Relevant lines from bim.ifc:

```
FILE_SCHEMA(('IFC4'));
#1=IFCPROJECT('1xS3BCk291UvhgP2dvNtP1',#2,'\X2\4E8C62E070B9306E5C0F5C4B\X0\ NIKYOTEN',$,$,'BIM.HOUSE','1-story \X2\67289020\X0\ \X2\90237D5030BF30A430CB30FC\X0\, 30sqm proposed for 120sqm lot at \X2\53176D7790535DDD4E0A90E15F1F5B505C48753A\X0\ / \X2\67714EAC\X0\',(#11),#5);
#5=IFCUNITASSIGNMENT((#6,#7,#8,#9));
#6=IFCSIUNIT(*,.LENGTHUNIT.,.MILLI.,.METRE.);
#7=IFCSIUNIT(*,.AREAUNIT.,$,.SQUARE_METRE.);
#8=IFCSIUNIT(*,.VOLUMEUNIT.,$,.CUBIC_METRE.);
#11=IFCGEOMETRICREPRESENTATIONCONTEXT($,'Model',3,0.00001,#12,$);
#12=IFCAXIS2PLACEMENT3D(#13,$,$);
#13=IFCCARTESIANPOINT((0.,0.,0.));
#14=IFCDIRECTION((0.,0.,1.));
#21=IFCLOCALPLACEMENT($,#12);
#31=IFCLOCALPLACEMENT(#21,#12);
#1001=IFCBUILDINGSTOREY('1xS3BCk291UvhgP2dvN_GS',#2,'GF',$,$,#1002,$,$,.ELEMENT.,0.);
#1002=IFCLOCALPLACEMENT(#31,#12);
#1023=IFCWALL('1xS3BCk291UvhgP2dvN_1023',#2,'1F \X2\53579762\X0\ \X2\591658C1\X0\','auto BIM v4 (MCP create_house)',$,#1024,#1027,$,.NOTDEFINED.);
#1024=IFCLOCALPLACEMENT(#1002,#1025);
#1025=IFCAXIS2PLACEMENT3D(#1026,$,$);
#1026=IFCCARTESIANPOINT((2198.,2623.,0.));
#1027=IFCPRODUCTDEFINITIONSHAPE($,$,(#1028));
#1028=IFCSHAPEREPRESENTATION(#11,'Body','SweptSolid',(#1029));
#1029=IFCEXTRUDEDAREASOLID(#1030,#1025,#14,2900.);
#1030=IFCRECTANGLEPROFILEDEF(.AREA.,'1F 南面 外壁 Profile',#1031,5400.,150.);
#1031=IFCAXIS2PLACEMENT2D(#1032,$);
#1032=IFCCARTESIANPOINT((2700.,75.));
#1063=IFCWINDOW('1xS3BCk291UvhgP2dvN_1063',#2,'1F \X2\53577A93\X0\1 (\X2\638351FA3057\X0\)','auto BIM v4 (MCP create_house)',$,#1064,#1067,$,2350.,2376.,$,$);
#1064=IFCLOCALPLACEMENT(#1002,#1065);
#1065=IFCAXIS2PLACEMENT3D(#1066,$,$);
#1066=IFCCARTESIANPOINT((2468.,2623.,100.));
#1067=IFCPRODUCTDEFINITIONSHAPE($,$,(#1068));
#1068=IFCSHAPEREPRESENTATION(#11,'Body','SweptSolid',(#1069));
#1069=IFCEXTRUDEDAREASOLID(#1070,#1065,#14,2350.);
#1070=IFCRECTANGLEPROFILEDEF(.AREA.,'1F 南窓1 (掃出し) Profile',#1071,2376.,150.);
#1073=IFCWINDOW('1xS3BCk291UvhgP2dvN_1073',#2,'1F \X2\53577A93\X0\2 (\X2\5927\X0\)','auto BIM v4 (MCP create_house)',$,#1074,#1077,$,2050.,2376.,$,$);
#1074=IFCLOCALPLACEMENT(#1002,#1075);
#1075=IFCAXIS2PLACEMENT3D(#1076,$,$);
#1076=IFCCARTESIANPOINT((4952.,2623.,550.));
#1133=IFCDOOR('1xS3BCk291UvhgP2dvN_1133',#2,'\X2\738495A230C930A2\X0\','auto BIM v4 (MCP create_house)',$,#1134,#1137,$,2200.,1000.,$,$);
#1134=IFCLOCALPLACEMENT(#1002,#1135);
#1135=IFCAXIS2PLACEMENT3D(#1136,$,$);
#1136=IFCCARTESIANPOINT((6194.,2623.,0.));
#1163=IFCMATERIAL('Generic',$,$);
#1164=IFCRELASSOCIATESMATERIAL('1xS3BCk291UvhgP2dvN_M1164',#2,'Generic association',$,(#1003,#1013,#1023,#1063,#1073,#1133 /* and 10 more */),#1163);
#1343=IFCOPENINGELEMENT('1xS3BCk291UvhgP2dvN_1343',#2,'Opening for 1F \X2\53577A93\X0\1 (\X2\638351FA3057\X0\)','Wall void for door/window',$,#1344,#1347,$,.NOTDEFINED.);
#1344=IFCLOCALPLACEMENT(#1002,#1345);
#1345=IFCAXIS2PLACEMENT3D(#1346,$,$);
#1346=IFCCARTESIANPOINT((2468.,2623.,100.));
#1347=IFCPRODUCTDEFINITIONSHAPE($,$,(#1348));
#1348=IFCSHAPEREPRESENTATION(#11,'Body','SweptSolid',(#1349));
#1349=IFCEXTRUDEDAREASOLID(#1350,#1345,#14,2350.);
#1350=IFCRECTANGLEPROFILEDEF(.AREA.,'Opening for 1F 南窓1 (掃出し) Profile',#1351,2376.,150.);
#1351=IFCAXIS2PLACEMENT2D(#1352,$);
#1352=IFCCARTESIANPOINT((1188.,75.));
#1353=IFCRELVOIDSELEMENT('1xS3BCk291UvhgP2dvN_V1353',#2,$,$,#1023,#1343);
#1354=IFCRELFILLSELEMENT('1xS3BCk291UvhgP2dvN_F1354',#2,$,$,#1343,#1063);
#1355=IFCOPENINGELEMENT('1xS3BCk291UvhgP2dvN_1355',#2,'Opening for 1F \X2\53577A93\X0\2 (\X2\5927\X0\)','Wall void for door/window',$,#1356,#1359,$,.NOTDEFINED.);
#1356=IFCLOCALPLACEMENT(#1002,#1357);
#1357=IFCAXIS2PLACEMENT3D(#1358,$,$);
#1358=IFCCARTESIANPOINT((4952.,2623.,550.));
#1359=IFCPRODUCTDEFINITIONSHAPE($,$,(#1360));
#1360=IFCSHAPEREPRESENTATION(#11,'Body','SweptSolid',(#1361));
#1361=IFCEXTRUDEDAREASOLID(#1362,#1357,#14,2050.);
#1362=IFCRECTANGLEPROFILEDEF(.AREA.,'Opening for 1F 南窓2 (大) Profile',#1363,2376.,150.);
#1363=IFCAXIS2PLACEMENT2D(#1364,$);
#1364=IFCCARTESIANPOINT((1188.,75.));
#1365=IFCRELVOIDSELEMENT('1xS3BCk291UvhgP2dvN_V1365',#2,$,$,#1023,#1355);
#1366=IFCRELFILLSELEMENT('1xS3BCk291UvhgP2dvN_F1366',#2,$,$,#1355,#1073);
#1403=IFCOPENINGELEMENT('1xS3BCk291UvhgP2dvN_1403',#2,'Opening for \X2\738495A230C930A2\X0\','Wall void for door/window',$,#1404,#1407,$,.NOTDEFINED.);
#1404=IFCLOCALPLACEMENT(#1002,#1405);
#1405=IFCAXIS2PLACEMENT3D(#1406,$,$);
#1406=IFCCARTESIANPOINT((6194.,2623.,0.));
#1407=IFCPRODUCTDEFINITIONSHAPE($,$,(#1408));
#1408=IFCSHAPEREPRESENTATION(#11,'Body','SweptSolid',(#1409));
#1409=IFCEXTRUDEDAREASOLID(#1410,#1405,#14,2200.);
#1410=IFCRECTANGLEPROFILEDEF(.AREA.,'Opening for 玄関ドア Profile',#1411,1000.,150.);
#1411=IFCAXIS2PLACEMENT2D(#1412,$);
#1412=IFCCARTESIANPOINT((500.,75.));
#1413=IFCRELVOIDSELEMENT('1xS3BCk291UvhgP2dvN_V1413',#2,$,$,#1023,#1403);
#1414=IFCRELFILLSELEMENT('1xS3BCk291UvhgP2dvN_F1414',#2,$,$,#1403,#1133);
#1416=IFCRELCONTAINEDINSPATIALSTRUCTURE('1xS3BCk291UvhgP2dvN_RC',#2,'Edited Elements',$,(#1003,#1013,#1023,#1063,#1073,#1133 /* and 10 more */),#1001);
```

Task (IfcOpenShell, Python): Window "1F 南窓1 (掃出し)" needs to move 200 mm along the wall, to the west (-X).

```python
import ifcopenshell
import ifcopenshell.api.geometry
import ifcopenshell.util.placement

model = ifcopenshell.open("bim.ifc")

window = model.by_id(1063)
opening = window.FillsVoids[0].RelatingOpeningElement
wall = opening.VoidsElements[0].RelatingBuildingElement

wall_matrix = ifcopenshell.util.placement.get_local_placement(wall.ObjectPlacement)
shift = wall_matrix[:3, 0] * -200.0
before = ifcopenshell.util.placement.get_local_placement(window.ObjectPlacement)[:3, 3].copy()

# The window is not placed relative to its opening, so move both.
for product in (opening, window):
    matrix = ifcopenshell.util.placement.get_local_placement(product.ObjectPlacement)
    matrix[:3, 3] += shift
    ifcopenshell.api.geometry.edit_object_placement(model, product=product, matrix=matrix, is_si=False)

after = ifcopenshell.util.placement.get_local_placement(window.ObjectPlacement)[:3, 3]
print("window moved by", (after - before).round(3) + 0.0)

model.write("bim_rev.ifc")
```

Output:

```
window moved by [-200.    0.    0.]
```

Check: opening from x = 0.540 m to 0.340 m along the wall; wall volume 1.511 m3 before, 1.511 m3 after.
